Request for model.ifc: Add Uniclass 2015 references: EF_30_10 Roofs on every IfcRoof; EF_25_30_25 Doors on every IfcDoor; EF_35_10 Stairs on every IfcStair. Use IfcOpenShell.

First a look at what the model holds.

```python
import ifcopenshell

model = ifcopenshell.open("model.ifc")
print(model.schema)
print("classifications:", [c.Name for c in model.by_type("IfcClassification")])
for ifc_class in ("IfcDoor", "IfcRoof", "IfcStair", "IfcWall", "IfcWindow"):
    print(ifc_class, len(model.by_type(ifc_class)))
```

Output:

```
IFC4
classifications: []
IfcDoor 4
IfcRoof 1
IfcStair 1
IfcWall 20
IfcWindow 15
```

```python
import ifcopenshell
import ifcopenshell.api.classification

model = ifcopenshell.open("model.ifc")

system = ifcopenshell.api.classification.add_classification(model, classification="Uniclass 2015")

codes = {
    "IfcRoof": ("EF_30_10", "Roofs"),
    "IfcDoor": ("EF_25_30_25", "Doors"),
    "IfcStair": ("EF_35_10", "Stairs"),
}
for ifc_class, (code, name) in codes.items():
    products = model.by_type(ifc_class)
    ifcopenshell.api.classification.add_reference(
        model, products=products, classification=system, identification=code, name=name
    )
    print(code, len(products))

model.write("model_rev.ifc")
```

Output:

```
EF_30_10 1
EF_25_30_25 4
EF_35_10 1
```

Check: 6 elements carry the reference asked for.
